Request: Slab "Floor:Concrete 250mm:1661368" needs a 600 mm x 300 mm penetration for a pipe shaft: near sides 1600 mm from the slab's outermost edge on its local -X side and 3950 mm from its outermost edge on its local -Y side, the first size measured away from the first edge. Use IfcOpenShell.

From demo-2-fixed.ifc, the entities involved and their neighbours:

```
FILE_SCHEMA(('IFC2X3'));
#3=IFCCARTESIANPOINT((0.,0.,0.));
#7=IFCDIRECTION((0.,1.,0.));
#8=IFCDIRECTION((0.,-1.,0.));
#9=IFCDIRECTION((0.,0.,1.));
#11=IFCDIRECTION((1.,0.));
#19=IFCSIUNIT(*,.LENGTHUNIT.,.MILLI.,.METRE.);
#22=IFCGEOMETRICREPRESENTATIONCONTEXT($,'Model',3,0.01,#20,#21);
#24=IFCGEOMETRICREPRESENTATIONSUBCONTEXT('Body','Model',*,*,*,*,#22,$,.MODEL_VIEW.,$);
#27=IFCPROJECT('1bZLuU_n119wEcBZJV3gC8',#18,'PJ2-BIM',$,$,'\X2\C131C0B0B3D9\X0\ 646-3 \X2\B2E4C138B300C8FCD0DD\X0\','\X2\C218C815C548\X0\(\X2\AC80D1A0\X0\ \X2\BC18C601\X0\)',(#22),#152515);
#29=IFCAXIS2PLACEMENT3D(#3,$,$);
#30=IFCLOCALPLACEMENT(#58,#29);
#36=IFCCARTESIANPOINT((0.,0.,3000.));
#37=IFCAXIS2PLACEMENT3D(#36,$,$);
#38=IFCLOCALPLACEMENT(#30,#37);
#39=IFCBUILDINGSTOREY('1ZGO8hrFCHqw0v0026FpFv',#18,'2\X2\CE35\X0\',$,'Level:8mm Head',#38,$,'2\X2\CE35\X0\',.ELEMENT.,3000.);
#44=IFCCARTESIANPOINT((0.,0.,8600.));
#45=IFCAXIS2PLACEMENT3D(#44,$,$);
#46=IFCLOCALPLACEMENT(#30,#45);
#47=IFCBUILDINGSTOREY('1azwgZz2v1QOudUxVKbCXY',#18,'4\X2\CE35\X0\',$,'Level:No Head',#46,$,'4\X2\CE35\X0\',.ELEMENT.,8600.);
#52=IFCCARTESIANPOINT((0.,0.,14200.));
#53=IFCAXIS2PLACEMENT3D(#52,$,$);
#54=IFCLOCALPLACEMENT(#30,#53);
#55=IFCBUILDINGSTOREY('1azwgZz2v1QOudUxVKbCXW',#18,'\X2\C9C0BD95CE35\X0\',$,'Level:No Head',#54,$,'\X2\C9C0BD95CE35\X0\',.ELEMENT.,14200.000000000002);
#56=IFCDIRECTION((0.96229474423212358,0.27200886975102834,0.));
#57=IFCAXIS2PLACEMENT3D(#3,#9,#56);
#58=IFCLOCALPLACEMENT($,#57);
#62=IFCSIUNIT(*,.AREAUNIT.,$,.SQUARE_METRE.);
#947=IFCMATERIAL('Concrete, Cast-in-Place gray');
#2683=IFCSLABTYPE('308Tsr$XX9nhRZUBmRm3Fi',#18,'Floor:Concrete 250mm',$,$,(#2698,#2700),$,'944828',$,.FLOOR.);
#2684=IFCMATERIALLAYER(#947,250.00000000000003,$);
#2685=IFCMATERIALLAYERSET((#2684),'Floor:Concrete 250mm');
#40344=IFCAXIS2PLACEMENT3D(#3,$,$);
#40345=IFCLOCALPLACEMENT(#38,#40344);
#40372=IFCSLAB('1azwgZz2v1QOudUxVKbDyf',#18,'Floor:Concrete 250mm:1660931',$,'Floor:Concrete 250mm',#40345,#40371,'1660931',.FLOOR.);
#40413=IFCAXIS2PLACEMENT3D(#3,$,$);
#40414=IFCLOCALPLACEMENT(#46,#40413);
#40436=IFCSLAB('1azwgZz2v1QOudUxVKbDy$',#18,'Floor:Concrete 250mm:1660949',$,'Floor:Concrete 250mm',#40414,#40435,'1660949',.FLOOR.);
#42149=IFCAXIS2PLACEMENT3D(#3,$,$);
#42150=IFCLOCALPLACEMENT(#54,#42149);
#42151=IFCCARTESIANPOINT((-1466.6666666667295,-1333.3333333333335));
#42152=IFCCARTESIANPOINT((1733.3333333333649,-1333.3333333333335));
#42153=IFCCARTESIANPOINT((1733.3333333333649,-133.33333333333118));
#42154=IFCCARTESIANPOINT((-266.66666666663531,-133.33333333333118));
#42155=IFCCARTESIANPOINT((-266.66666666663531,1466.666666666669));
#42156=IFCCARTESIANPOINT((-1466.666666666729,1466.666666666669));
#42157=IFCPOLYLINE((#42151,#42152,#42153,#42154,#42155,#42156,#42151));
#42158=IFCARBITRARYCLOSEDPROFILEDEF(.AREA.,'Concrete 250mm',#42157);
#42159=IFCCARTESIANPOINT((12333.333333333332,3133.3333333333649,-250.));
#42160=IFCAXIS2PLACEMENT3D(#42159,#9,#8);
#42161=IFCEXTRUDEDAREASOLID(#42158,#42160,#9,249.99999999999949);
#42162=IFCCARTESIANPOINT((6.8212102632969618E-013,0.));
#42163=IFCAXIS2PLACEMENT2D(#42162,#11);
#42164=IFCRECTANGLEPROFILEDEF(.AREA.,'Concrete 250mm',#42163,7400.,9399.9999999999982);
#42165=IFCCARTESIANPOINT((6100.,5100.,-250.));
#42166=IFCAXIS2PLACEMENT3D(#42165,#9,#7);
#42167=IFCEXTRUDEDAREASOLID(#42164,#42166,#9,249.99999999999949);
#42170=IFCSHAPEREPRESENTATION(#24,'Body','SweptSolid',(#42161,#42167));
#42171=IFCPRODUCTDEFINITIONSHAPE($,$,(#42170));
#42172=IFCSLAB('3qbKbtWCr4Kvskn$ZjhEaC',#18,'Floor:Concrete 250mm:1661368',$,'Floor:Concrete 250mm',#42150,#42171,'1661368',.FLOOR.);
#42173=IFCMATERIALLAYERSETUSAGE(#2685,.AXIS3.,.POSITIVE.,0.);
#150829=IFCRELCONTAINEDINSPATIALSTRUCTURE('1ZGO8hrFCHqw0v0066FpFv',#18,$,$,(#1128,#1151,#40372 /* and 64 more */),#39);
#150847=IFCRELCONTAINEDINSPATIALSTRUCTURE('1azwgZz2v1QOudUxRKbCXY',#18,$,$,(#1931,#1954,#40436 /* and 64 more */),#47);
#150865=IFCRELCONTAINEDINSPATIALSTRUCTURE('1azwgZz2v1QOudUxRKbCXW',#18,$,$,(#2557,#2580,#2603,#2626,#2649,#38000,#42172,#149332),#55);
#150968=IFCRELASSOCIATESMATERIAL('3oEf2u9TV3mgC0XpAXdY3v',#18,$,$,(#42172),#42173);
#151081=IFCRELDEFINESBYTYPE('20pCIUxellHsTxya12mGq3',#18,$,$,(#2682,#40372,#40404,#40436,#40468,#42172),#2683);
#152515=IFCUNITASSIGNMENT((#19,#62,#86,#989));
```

```python
import numpy as np
import ifcopenshell
import ifcopenshell.api.feature
import ifcopenshell.api.geometry
import ifcopenshell.api.root
import ifcopenshell.geom
import ifcopenshell.util.placement
import ifcopenshell.util.representation
import ifcopenshell.util.shape
import ifcopenshell.util.unit

model = ifcopenshell.open("demo-2-fixed.ifc")
unit_scale = ifcopenshell.util.unit.calculate_unit_scale(model)
settings = ifcopenshell.geom.settings()


def volume(element):
    """Net volume in cubic metres, openings subtracted."""
    shape = ifcopenshell.geom.create_shape(settings, element)
    return ifcopenshell.util.shape.get_volume(shape.geometry)


slab = model.by_guid("3qbKbtWCr4Kvskn$ZjhEaC")
before = volume(slab)

# Extent in the slab's own axes, in metres. The edges named are its -X and -Y sides.
slab_shape = ifcopenshell.geom.create_shape(settings, slab)
vertices = ifcopenshell.util.shape.get_vertices(slab_shape.geometry)
x_min, y_min, bottom = vertices.min(axis=0)
top = vertices[:, 2].max()

opening = ifcopenshell.api.root.create_entity(model, ifc_class="IfcOpeningElement", name="Pipe shaft opening")
context = ifcopenshell.util.representation.get_context(model, "Model", "Body", "MODEL_VIEW")
width, depth = 0.6, 0.3
outline = [(0.0, 0.0), (width, 0.0), (width, depth), (0.0, depth), (0.0, 0.0)]
# Overshoot both faces by 50 mm so the cut is clean.
shape = ifcopenshell.api.geometry.add_slab_representation(
    model, context=context, depth=top - bottom + 0.1, polyline=outline
)
ifcopenshell.api.geometry.assign_representation(model, product=opening, representation=shape)

matrix = ifcopenshell.util.placement.get_local_placement(slab.ObjectPlacement)
matrix[:, 3] = matrix @ np.append(np.array([x_min + 1.6, y_min + 3.95, bottom - 0.05]) / unit_scale, 1.0)
ifcopenshell.api.geometry.edit_object_placement(model, product=opening, matrix=matrix, is_si=False)
ifcopenshell.api.feature.add_feature(model, feature=opening, element=slab)

after = volume(slab)

print(f"slab volume {before:.3f} -> {after:.3f} m3")

model.write("demo-2-fixed_updated.ifc")
```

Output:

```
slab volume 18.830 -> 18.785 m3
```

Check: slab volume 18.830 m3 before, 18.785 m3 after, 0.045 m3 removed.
